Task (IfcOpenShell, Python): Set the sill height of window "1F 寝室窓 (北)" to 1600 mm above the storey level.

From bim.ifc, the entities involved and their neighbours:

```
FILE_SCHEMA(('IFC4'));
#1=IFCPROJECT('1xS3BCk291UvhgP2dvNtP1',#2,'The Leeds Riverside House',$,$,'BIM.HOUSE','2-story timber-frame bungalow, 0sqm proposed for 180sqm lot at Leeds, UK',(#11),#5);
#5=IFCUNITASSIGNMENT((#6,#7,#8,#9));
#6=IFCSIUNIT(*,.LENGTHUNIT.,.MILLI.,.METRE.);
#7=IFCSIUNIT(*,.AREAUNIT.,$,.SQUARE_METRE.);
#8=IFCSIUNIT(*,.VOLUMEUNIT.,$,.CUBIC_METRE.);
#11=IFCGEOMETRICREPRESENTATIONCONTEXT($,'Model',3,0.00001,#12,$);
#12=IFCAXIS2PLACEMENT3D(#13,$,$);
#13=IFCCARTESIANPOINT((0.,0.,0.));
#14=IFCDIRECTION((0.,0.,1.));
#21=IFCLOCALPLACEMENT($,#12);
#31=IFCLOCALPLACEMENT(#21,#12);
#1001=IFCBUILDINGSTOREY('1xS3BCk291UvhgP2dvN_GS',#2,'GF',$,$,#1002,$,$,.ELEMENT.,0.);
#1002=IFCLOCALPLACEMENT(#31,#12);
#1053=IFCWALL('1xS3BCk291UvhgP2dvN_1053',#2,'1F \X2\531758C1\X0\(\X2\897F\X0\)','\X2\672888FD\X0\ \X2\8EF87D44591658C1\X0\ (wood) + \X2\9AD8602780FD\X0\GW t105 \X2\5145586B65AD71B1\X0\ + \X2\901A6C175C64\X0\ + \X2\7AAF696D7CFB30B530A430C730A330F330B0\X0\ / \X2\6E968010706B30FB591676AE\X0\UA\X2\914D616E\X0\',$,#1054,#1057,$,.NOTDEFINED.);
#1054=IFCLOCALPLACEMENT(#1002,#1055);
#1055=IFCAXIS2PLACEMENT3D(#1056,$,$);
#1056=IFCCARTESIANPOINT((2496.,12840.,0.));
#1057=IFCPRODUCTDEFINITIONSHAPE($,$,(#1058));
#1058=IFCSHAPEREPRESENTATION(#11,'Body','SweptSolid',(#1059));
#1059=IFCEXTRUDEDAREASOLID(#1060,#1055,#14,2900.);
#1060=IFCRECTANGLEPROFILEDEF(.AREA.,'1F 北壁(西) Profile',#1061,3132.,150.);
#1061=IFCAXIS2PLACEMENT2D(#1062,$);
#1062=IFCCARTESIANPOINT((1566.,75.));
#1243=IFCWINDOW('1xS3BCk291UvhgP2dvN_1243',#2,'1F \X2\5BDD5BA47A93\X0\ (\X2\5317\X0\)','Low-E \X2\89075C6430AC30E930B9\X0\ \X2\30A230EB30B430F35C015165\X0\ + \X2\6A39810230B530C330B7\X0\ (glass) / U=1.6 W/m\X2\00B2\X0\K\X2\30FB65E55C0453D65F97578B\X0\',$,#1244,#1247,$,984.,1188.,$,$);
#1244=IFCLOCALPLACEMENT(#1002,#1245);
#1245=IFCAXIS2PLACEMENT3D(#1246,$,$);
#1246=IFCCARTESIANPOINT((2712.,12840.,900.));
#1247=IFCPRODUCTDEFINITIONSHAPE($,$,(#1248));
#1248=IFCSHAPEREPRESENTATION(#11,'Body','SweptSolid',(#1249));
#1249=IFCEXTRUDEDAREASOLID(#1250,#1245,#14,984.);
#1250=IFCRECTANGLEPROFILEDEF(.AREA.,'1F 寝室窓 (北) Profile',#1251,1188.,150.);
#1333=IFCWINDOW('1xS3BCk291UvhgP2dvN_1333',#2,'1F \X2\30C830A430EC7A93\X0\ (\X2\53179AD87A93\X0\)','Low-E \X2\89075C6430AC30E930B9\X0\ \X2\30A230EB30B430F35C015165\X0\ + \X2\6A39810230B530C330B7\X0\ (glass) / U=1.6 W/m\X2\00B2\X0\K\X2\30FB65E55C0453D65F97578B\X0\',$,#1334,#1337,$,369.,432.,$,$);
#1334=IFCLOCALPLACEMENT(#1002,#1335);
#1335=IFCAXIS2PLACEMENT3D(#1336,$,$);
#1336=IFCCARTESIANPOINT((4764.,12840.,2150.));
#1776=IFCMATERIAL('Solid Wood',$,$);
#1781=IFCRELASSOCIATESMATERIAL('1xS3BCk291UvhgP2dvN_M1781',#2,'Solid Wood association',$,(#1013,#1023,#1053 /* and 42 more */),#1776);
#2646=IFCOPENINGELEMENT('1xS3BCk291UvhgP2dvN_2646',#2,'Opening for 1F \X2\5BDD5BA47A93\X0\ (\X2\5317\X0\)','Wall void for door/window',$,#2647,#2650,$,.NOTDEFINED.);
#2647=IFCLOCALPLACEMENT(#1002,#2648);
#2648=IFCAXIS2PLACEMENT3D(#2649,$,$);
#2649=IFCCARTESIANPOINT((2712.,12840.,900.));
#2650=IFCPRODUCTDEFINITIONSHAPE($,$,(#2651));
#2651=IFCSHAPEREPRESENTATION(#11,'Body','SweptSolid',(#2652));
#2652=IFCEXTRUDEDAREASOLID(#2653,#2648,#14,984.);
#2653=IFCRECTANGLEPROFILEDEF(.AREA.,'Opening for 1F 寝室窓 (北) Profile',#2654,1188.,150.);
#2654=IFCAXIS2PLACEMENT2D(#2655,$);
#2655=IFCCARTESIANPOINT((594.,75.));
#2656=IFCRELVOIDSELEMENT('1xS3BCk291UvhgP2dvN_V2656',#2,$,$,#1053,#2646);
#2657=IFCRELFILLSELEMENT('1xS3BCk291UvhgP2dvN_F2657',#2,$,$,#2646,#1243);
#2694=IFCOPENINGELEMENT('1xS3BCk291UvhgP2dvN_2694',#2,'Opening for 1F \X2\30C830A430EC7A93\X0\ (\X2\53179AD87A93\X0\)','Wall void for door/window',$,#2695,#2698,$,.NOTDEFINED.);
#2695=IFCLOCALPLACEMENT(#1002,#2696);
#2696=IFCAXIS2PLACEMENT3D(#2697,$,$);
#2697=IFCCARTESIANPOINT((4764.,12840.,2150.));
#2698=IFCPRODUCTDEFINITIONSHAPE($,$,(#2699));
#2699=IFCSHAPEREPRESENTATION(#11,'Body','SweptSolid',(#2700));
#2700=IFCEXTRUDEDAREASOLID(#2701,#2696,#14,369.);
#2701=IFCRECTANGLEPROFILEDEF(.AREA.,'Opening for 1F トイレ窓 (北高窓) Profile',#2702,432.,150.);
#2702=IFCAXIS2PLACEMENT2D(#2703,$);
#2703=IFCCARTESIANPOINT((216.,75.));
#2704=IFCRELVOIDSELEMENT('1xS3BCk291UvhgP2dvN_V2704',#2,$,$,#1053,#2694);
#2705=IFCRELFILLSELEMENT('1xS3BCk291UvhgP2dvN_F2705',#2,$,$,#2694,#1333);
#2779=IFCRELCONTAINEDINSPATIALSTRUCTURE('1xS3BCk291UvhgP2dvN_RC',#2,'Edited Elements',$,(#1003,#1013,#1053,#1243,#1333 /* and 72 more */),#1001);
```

```python
import numpy as np
import ifcopenshell
import ifcopenshell.api.geometry
import ifcopenshell.geom
import ifcopenshell.util.element
import ifcopenshell.util.placement
import ifcopenshell.util.shape
import ifcopenshell.util.unit

model = ifcopenshell.open("bim.ifc")
unit_scale = ifcopenshell.util.unit.calculate_unit_scale(model)

window = model.by_id(1243)
opening = window.FillsVoids[0].RelatingOpeningElement
storey = ifcopenshell.util.element.get_container(window, ifc_class="IfcBuildingStorey")
level = ifcopenshell.util.placement.get_local_placement(storey.ObjectPlacement)[2, 3]

# The opening's origin need not be at the sill, so measure its lowest point.
shape = ifcopenshell.geom.create_shape(ifcopenshell.geom.settings(), opening)
bottom = ifcopenshell.util.shape.get_shape_bottom_elevation(shape, shape.geometry) / unit_scale
dz = level + 1.6 / unit_scale - bottom

shift = np.array([0.0, 0.0, dz])
# The window is not placed relative to its opening, so move both.
for product in (opening, window):
    matrix = ifcopenshell.util.placement.get_local_placement(product.ObjectPlacement)
    matrix[:3, 3] += shift
    ifcopenshell.api.geometry.edit_object_placement(model, product=product, matrix=matrix, is_si=False)

print(f"moved by {dz * unit_scale:+.3f} m")

model.write("bim_v2.ifc")
```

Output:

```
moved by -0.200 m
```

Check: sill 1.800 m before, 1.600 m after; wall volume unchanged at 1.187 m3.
